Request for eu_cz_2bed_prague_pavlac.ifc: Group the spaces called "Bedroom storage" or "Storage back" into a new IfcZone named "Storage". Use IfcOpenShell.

First a look at what the model holds.

```python
import ifcopenshell

model = ifcopenshell.open("eu_cz_2bed_prague_pavlac.ifc")
print(model.schema)
seen = {}
for space in model.by_type("IfcSpace"):
    seen[space.LongName] = seen.get(space.LongName, 0) + 1
for name, count in sorted(seen.items(), key=str):
    print(count, "x", name)
print("zones:", [z.Name for z in model.by_type("IfcZone")][:20])
```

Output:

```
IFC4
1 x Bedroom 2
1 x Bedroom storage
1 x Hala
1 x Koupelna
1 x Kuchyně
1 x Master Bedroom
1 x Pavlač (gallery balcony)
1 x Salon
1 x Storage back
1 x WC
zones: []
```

```python
import ifcopenshell
import ifcopenshell.api.group
import ifcopenshell.api.root

model = ifcopenshell.open("eu_cz_2bed_prague_pavlac.ifc")

names = {"Bedroom storage", "Storage back"}
spaces = [s for s in model.by_type("IfcSpace") if s.LongName in names]

zone = ifcopenshell.api.root.create_entity(model, ifc_class="IfcZone", name="Storage")
ifcopenshell.api.group.assign_group(model, products=spaces, group=zone)
print(len(spaces), "spaces in", zone.Name)

model.write("eu_cz_2bed_prague_pavlac_v2.ifc")
```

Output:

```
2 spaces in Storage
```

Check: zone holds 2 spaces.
